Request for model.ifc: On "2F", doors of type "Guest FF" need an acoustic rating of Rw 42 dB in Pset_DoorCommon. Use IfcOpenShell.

First a look at what the model holds.

```python
import ifcopenshell
import ifcopenshell.util.element

model = ifcopenshell.open("model.ifc")
print(model.schema)
storey = next(s for s in model.by_type("IfcBuildingStorey") if s.Name == "2F")
doors = [e for e in ifcopenshell.util.element.get_decomposition(storey) if e.is_a("IfcDoor")]
seen = {}
for e in doors:
    element_type = ifcopenshell.util.element.get_type(e)
    key = (element_type.Name if element_type != e and element_type else None, ifcopenshell.util.element.get_pset(e, "Pset_DoorCommon", "AcousticRating"))
    seen[key] = seen.get(key, 0) + 1
for (name, value), count in sorted(seen.items(), key=str):
    print(count, "x", name, "|", value)
```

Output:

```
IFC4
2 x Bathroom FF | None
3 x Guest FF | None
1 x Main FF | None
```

```python
import ifcopenshell
import ifcopenshell.api.pset
import ifcopenshell.util.element

model = ifcopenshell.open("model.ifc")

storey = next(s for s in model.by_type("IfcBuildingStorey") if s.Name == "2F")
doors = [e for e in ifcopenshell.util.element.get_decomposition(storey) if e.is_a("IfcDoor")]

count = 0
for e in doors:
    element_type = ifcopenshell.util.element.get_type(e)
    if element_type in (None, e) or element_type.Name != "Guest FF":
        continue
    # add_pset returns the element's existing set when there is one.
    pset = ifcopenshell.api.pset.add_pset(model, product=e, name="Pset_DoorCommon")
    ifcopenshell.api.pset.edit_pset(model, pset=pset, properties={"AcousticRating": "Rw 42 dB"})
    count += 1

print(count, "doors updated")

model.write("model_edited.ifc")
```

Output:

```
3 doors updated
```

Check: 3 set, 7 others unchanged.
